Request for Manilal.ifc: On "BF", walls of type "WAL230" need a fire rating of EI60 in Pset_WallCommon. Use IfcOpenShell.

First a look at what the model holds.

```python
import ifcopenshell
import ifcopenshell.util.element

model = ifcopenshell.open("Manilal.ifc")
print(model.schema)
storey = next(s for s in model.by_type("IfcBuildingStorey") if s.Name == "BF")
walls = [e for e in ifcopenshell.util.element.get_decomposition(storey) if e.is_a("IfcWall")]
seen = {}
for e in walls:
    element_type = ifcopenshell.util.element.get_type(e)
    key = (element_type.Name if element_type != e and element_type else None, ifcopenshell.util.element.get_pset(e, "Pset_WallCommon", "FireRating"))
    seen[key] = seen.get(key, 0) + 1
for (name, value), count in sorted(seen.items(), key=str):
    print(count, "x", name, "|", value)
```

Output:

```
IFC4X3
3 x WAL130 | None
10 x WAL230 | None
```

```python
import ifcopenshell
import ifcopenshell.api.pset
import ifcopenshell.util.element

model = ifcopenshell.open("Manilal.ifc")

storey = next(s for s in model.by_type("IfcBuildingStorey") if s.Name == "BF")
walls = [e for e in ifcopenshell.util.element.get_decomposition(storey) if e.is_a("IfcWall")]

count = 0
for e in walls:
    element_type = ifcopenshell.util.element.get_type(e)
    if element_type in (None, e) or element_type.Name != "WAL230":
        continue
    # add_pset returns the element's existing set when there is one.
    pset = ifcopenshell.api.pset.add_pset(model, product=e, name="Pset_WallCommon")
    ifcopenshell.api.pset.edit_pset(model, pset=pset, properties={"FireRating": "EI60"})
    count += 1

print(count, "walls updated")

model.write("Manilal_rev.ifc")
```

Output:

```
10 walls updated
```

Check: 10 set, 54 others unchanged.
